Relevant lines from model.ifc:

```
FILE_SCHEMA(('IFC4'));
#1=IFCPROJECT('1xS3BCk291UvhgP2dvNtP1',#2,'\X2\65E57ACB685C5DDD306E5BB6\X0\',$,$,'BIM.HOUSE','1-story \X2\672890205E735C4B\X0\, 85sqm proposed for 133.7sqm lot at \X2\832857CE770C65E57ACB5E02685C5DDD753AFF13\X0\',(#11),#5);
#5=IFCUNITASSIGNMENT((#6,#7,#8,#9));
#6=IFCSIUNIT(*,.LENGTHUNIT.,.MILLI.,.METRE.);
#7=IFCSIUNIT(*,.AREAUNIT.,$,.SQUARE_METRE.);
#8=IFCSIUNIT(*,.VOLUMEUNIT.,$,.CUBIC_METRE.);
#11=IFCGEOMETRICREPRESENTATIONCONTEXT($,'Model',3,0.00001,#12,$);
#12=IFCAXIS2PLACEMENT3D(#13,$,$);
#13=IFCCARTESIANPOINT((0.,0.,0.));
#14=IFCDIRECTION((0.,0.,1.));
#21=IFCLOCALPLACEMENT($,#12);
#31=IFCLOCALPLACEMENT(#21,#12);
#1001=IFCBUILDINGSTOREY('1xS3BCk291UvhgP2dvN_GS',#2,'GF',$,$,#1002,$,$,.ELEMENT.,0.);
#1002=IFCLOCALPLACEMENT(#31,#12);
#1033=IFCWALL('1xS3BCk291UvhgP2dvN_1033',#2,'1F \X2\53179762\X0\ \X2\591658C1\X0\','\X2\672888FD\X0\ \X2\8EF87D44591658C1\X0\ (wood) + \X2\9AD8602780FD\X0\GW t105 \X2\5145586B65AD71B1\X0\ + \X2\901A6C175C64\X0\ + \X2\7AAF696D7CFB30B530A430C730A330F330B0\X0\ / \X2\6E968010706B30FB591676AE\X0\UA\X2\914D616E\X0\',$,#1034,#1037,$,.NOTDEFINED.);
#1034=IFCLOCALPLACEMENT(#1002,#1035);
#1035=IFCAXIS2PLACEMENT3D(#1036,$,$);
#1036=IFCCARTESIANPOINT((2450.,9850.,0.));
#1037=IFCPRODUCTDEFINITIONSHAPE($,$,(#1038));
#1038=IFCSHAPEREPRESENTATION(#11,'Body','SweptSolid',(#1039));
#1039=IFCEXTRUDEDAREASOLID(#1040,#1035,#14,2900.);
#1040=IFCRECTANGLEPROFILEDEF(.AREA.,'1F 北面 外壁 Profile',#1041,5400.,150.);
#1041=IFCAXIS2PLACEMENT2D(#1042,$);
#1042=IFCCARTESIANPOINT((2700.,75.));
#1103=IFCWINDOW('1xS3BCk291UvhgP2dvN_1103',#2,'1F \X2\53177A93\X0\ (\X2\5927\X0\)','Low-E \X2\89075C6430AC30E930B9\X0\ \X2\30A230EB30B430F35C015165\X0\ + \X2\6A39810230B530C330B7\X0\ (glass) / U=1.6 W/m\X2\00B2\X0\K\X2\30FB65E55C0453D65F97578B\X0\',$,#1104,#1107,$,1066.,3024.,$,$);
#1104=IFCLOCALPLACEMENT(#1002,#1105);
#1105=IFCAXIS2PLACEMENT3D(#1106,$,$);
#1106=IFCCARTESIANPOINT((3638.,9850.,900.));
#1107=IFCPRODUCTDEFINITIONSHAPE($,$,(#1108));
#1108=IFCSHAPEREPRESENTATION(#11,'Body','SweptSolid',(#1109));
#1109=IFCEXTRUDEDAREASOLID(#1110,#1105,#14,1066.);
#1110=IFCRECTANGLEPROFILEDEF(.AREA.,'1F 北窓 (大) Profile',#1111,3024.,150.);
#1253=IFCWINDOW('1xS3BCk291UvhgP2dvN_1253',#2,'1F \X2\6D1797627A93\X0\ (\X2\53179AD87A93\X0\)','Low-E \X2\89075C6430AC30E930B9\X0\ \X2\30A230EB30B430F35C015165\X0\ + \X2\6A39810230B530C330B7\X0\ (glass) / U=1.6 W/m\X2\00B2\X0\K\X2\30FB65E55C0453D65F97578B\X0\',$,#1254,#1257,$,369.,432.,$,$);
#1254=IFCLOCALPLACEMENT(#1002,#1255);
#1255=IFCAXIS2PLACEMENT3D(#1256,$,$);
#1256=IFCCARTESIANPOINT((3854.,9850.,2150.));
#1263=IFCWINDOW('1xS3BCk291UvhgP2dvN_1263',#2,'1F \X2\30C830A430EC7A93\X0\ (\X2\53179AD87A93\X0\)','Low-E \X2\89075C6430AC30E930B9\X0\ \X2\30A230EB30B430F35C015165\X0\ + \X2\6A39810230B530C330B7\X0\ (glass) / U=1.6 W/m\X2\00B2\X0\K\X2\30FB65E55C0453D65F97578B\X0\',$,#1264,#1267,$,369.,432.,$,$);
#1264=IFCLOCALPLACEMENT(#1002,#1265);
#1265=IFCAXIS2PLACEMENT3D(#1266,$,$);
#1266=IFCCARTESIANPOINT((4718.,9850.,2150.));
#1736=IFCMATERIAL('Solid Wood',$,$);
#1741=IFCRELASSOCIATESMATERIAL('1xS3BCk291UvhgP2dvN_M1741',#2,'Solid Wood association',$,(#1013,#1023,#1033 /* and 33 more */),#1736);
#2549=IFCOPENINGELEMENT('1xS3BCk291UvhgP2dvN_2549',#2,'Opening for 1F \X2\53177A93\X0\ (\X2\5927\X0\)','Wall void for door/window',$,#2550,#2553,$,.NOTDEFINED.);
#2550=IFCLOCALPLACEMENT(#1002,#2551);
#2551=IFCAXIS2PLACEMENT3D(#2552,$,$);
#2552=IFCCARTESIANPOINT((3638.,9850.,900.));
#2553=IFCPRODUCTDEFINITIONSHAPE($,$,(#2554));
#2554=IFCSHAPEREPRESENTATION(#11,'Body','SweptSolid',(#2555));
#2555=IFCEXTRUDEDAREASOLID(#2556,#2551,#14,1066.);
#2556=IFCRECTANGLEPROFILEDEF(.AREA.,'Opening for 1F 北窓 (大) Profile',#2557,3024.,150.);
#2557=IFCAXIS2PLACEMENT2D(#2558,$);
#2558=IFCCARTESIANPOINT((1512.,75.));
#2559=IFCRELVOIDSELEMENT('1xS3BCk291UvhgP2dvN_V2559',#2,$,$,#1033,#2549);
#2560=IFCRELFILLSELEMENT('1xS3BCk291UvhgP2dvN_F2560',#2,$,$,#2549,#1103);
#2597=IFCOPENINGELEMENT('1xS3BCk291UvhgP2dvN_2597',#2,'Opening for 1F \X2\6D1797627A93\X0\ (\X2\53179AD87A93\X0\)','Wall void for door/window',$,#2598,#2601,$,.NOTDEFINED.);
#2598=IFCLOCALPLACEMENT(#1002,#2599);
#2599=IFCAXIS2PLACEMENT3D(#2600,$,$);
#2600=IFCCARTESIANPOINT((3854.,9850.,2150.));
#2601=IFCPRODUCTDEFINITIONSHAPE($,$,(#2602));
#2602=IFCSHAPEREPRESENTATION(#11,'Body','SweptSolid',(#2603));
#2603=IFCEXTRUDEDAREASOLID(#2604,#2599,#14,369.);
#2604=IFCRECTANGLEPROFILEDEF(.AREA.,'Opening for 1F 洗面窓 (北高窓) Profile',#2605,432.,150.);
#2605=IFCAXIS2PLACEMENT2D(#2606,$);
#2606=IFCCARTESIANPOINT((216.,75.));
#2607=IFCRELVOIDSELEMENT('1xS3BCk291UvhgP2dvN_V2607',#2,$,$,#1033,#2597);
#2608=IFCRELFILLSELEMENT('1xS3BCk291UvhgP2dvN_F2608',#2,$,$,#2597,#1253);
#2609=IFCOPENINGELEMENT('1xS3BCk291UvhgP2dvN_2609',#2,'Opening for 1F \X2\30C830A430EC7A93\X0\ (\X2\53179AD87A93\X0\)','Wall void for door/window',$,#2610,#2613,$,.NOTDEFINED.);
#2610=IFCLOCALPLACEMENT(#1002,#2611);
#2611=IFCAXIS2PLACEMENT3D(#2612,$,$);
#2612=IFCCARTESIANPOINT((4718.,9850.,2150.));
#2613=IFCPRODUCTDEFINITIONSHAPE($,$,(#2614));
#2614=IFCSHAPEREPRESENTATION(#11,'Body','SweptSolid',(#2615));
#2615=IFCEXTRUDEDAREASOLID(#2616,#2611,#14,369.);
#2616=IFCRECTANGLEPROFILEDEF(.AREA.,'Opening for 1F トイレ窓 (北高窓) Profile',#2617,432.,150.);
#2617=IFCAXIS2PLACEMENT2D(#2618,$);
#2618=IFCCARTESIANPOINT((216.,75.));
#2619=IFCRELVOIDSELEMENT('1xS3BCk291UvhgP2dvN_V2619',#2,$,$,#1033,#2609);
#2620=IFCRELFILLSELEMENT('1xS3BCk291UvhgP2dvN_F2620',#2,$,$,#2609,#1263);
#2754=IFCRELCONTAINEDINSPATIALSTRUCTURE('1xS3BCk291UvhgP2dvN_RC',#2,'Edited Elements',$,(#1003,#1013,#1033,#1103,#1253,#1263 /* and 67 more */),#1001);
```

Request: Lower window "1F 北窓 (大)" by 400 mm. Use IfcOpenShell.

```python
import numpy as np
import ifcopenshell
import ifcopenshell.api.geometry
import ifcopenshell.util.placement
import ifcopenshell.util.unit

model = ifcopenshell.open("model.ifc")
unit_scale = ifcopenshell.util.unit.calculate_unit_scale(model)

window = model.by_guid("1xS3BCk291UvhgP2dvN_1103")
opening = window.FillsVoids[0].RelatingOpeningElement
dz = -400.0

shift = np.array([0.0, 0.0, dz])
# The window is not placed relative to its opening, so move both.
for product in (opening, window):
    matrix = ifcopenshell.util.placement.get_local_placement(product.ObjectPlacement)
    matrix[:3, 3] += shift
    ifcopenshell.api.geometry.edit_object_placement(model, product=product, matrix=matrix, is_si=False)

print(f"moved by {dz * unit_scale:+.3f} m")

model.write("model_updated.ifc")
```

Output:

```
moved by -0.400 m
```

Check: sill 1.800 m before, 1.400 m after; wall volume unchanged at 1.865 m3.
